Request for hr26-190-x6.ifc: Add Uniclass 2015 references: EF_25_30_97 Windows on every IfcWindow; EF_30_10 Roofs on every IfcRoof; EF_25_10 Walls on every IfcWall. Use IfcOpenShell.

First a look at what the model holds.

```python
import ifcopenshell

model = ifcopenshell.open("hr26-190-x6.ifc")
print(model.schema)
print("classifications:", [c.Name for c in model.by_type("IfcClassification")])
for ifc_class in ("IfcDoor", "IfcRoof", "IfcStair", "IfcWall", "IfcWindow"):
    print(ifc_class, len(model.by_type(ifc_class)))
```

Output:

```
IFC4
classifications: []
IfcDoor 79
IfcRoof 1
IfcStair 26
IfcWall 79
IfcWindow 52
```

```python
import ifcopenshell
import ifcopenshell.api.classification

model = ifcopenshell.open("hr26-190-x6.ifc")

system = ifcopenshell.api.classification.add_classification(model, classification="Uniclass 2015")

codes = {
    "IfcWindow": ("EF_25_30_97", "Windows"),
    "IfcRoof": ("EF_30_10", "Roofs"),
    "IfcWall": ("EF_25_10", "Walls"),
}
for ifc_class, (code, name) in codes.items():
    products = model.by_type(ifc_class)
    ifcopenshell.api.classification.add_reference(
        model, products=products, classification=system, identification=code, name=name
    )
    print(code, len(products))

model.write("hr26-190-x6_updated.ifc")
```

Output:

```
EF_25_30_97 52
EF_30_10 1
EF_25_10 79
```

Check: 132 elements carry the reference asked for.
